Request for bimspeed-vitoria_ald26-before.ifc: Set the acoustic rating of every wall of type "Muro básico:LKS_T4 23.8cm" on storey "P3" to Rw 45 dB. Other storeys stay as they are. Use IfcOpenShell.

First a look at what the model holds.

```python
import ifcopenshell
import ifcopenshell.util.element

model = ifcopenshell.open("bimspeed-vitoria_ald26-before.ifc")
print(model.schema)
storey = next(s for s in model.by_type("IfcBuildingStorey") if s.Name == "P3")
walls = [e for e in ifcopenshell.util.element.get_decomposition(storey) if e.is_a("IfcWall")]
seen = {}
for e in walls:
    element_type = ifcopenshell.util.element.get_type(e)
    key = (element_type.Name if element_type != e and element_type else None, ifcopenshell.util.element.get_pset(e, "Pset_WallCommon", "AcousticRating"))
    seen[key] = seen.get(key, 0) + 1
for (name, value), count in sorted(seen.items(), key=str):
    print(count, "x", name, "|", value)
```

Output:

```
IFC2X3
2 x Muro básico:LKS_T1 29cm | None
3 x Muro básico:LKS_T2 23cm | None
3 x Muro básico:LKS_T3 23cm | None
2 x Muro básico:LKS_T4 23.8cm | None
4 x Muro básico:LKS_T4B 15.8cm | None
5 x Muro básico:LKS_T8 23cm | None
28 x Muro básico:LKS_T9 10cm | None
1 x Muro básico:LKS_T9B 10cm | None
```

```python
import ifcopenshell
import ifcopenshell.api.pset
import ifcopenshell.util.element

model = ifcopenshell.open("bimspeed-vitoria_ald26-before.ifc")

storey = next(s for s in model.by_type("IfcBuildingStorey") if s.Name == "P3")
walls = [e for e in ifcopenshell.util.element.get_decomposition(storey) if e.is_a("IfcWall")]

count = 0
for e in walls:
    element_type = ifcopenshell.util.element.get_type(e)
    if element_type in (None, e) or element_type.Name != "Muro básico:LKS_T4 23.8cm":
        continue
    # add_pset returns the element's existing set when there is one.
    pset = ifcopenshell.api.pset.add_pset(model, product=e, name="Pset_WallCommon")
    ifcopenshell.api.pset.edit_pset(model, pset=pset, properties={"AcousticRating": "Rw 45 dB"})
    count += 1

print(count, "walls updated")

model.write("bimspeed-vitoria_ald26-before_v2.ifc")
```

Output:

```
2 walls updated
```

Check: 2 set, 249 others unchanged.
